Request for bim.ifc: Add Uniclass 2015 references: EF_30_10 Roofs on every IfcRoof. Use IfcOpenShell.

First a look at what the model holds.

```python
import ifcopenshell

model = ifcopenshell.open("bim.ifc")
print(model.schema)
print("classifications:", [c.Name for c in model.by_type("IfcClassification")])
for ifc_class in ("IfcDoor", "IfcRoof", "IfcStair", "IfcWall", "IfcWindow"):
    print(ifc_class, len(model.by_type(ifc_class)))
```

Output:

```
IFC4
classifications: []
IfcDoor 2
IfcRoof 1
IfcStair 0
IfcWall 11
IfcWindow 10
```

```python
import ifcopenshell
import ifcopenshell.api.classification

model = ifcopenshell.open("bim.ifc")

system = ifcopenshell.api.classification.add_classification(model, classification="Uniclass 2015")

codes = {
    "IfcRoof": ("EF_30_10", "Roofs"),
}
for ifc_class, (code, name) in codes.items():
    products = model.by_type(ifc_class)
    ifcopenshell.api.classification.add_reference(
        model, products=products, classification=system, identification=code, name=name
    )
    print(code, len(products))

model.write("bim_edited.ifc")
```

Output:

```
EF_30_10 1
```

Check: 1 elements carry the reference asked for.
